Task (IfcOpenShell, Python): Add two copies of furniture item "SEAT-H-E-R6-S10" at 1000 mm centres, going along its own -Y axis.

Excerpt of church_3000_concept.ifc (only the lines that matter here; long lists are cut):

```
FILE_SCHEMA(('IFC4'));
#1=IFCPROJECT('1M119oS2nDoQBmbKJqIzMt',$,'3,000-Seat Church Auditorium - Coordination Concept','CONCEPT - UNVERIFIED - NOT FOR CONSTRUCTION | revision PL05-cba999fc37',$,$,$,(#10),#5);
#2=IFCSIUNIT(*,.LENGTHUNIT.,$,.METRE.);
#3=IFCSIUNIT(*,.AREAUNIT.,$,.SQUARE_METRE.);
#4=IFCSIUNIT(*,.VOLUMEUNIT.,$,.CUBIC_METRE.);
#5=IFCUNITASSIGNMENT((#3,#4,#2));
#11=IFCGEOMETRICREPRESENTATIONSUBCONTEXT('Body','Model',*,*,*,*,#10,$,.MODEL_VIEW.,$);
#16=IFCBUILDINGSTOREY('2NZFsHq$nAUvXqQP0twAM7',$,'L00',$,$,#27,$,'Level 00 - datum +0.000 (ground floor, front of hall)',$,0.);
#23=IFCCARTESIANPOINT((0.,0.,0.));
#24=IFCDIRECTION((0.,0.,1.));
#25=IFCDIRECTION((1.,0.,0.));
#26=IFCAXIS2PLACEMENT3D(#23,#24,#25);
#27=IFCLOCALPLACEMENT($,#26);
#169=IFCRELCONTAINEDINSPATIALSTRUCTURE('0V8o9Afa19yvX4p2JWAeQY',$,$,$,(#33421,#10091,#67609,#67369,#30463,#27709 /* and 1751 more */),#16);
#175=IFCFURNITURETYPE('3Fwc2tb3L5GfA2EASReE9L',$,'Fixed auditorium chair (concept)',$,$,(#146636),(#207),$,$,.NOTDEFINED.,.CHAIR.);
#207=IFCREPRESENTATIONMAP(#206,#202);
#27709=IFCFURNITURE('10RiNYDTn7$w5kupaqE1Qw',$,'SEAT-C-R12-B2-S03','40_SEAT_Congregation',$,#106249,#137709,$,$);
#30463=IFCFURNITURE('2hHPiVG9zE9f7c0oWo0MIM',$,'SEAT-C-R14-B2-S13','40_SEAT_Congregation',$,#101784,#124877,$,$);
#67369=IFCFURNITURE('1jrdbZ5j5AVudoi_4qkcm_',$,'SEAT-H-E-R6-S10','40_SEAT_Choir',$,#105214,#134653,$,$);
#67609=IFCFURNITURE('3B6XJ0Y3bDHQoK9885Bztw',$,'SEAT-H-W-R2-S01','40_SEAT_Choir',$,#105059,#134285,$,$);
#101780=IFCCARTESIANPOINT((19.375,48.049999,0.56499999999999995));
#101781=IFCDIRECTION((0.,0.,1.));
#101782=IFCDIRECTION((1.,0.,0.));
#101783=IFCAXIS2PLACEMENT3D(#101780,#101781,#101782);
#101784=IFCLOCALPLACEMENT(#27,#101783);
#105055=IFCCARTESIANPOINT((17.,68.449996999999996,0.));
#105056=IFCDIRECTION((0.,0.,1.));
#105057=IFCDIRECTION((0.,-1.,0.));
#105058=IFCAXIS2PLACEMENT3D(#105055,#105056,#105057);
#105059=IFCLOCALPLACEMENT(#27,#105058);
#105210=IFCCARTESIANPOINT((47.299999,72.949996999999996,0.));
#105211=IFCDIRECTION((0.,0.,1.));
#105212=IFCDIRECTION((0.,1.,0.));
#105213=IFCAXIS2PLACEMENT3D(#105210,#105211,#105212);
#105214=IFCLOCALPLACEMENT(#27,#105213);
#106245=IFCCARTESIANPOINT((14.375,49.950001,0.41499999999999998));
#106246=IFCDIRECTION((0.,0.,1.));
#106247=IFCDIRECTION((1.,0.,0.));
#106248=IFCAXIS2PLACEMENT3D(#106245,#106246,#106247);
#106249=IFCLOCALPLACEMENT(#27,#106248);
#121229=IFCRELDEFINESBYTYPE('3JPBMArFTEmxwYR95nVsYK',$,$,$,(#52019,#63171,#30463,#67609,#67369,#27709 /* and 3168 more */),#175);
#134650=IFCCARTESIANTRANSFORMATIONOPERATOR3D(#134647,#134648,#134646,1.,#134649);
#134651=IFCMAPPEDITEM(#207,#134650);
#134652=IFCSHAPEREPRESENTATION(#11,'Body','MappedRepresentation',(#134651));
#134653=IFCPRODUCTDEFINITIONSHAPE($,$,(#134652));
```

```python
import ifcopenshell
import ifcopenshell.api.geometry
import ifcopenshell.api.root
import ifcopenshell.util.element
import ifcopenshell.util.placement

model = ifcopenshell.open("church_3000_concept.ifc")

source = model.by_guid("1jrdbZ5j5AVudoi_4qkcm_")
base = ifcopenshell.util.placement.get_local_placement(source.ObjectPlacement)
step = -base[:3, 1] * 1.0

for i in range(1, 3):
    copy = ifcopenshell.api.root.copy_class(model, product=source)
    copy.Representation = ifcopenshell.util.element.copy_deep(
        model, source.Representation, exclude=["IfcGeometricRepresentationContext", "IfcRepresentationMap"]
    )
    matrix = base.copy()
    matrix[:3, 3] += i * step
    print("added at", matrix[:3, 3].round(3) + 0.0)
    ifcopenshell.api.geometry.edit_object_placement(model, product=copy, matrix=matrix, is_si=False)

model.write("church_3000_concept_rev.ifc")
```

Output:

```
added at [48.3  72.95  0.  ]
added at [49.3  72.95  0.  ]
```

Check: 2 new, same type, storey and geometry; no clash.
